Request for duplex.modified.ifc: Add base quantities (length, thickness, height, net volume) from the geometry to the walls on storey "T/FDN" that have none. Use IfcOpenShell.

First a look at what the model holds.

```python
import ifcopenshell
import ifcopenshell.util.element
import ifcopenshell.util.unit

model = ifcopenshell.open("duplex.modified.ifc")
print(model.schema)
for unit_type in ("LENGTHUNIT", "AREAUNIT", "VOLUMEUNIT"):
    print(unit_type, ifcopenshell.util.unit.calculate_unit_scale(model, unit_type))
storey = next(s for s in model.by_type("IfcBuildingStorey") if s.Name == "T/FDN")
walls = [e for e in ifcopenshell.util.element.get_decomposition(storey) if e.is_a("IfcWall")]
for e in sorted(walls, key=lambda e: e.id()):
    print(e.id(), e.is_a(), e.Name, list(ifcopenshell.util.element.get_psets(e, qtos_only=True)), sep=" | ")
```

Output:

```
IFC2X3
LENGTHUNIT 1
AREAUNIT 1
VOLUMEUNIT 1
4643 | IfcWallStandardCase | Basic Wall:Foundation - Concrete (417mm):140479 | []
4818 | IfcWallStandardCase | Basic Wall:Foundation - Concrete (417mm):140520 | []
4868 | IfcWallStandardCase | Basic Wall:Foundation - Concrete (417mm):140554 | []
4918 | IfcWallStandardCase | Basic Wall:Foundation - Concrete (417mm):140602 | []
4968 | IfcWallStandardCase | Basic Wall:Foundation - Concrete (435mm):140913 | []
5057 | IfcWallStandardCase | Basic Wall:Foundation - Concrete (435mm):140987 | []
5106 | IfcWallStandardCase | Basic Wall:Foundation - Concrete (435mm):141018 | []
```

```python
import ifcopenshell
import ifcopenshell.api.pset
import ifcopenshell.geom
import ifcopenshell.util.element
import ifcopenshell.util.shape
import ifcopenshell.util.unit

model = ifcopenshell.open("duplex.modified.ifc")
unit_scale = ifcopenshell.util.unit.calculate_unit_scale(model)
volume_scale = ifcopenshell.util.unit.calculate_unit_scale(model, "VOLUMEUNIT")
settings = ifcopenshell.geom.settings()

storey = next(s for s in model.by_type("IfcBuildingStorey") if s.Name == "T/FDN")
walls = [e for e in ifcopenshell.util.element.get_decomposition(storey) if e.is_a("IfcWall")]

for e in sorted(walls, key=lambda e: e.id()):
    if ifcopenshell.util.element.get_psets(e, qtos_only=True, should_inherit=False):
        continue
    # Geometry comes back in metres, in the element's own axes.
    shape = ifcopenshell.geom.create_shape(settings, e)
    values = {
        "Length": ifcopenshell.util.shape.get_x(shape.geometry) / unit_scale,
        "Width": ifcopenshell.util.shape.get_y(shape.geometry) / unit_scale,
        "Height": ifcopenshell.util.shape.get_z(shape.geometry) / unit_scale,
        "NetVolume": ifcopenshell.util.shape.get_volume(shape.geometry) / volume_scale,
    }
    qto = ifcopenshell.api.pset.add_qto(model, product=e, name="BaseQuantities")
    ifcopenshell.api.pset.edit_qto(model, qto=qto, properties=values)
    print(e.id(), {k: round(v, 3) for k, v in values.items()})

model.write("duplex.modified-out.ifc")
```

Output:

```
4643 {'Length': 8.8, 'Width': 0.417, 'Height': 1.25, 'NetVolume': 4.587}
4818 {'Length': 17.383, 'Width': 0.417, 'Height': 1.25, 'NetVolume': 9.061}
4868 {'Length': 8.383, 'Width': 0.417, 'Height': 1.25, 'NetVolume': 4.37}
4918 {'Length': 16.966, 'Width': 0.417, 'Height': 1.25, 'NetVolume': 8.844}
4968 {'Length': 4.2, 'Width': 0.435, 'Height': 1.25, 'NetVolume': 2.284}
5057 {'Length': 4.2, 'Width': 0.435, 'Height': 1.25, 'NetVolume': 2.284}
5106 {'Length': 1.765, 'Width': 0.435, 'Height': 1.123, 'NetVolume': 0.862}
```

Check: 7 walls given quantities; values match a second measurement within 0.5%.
